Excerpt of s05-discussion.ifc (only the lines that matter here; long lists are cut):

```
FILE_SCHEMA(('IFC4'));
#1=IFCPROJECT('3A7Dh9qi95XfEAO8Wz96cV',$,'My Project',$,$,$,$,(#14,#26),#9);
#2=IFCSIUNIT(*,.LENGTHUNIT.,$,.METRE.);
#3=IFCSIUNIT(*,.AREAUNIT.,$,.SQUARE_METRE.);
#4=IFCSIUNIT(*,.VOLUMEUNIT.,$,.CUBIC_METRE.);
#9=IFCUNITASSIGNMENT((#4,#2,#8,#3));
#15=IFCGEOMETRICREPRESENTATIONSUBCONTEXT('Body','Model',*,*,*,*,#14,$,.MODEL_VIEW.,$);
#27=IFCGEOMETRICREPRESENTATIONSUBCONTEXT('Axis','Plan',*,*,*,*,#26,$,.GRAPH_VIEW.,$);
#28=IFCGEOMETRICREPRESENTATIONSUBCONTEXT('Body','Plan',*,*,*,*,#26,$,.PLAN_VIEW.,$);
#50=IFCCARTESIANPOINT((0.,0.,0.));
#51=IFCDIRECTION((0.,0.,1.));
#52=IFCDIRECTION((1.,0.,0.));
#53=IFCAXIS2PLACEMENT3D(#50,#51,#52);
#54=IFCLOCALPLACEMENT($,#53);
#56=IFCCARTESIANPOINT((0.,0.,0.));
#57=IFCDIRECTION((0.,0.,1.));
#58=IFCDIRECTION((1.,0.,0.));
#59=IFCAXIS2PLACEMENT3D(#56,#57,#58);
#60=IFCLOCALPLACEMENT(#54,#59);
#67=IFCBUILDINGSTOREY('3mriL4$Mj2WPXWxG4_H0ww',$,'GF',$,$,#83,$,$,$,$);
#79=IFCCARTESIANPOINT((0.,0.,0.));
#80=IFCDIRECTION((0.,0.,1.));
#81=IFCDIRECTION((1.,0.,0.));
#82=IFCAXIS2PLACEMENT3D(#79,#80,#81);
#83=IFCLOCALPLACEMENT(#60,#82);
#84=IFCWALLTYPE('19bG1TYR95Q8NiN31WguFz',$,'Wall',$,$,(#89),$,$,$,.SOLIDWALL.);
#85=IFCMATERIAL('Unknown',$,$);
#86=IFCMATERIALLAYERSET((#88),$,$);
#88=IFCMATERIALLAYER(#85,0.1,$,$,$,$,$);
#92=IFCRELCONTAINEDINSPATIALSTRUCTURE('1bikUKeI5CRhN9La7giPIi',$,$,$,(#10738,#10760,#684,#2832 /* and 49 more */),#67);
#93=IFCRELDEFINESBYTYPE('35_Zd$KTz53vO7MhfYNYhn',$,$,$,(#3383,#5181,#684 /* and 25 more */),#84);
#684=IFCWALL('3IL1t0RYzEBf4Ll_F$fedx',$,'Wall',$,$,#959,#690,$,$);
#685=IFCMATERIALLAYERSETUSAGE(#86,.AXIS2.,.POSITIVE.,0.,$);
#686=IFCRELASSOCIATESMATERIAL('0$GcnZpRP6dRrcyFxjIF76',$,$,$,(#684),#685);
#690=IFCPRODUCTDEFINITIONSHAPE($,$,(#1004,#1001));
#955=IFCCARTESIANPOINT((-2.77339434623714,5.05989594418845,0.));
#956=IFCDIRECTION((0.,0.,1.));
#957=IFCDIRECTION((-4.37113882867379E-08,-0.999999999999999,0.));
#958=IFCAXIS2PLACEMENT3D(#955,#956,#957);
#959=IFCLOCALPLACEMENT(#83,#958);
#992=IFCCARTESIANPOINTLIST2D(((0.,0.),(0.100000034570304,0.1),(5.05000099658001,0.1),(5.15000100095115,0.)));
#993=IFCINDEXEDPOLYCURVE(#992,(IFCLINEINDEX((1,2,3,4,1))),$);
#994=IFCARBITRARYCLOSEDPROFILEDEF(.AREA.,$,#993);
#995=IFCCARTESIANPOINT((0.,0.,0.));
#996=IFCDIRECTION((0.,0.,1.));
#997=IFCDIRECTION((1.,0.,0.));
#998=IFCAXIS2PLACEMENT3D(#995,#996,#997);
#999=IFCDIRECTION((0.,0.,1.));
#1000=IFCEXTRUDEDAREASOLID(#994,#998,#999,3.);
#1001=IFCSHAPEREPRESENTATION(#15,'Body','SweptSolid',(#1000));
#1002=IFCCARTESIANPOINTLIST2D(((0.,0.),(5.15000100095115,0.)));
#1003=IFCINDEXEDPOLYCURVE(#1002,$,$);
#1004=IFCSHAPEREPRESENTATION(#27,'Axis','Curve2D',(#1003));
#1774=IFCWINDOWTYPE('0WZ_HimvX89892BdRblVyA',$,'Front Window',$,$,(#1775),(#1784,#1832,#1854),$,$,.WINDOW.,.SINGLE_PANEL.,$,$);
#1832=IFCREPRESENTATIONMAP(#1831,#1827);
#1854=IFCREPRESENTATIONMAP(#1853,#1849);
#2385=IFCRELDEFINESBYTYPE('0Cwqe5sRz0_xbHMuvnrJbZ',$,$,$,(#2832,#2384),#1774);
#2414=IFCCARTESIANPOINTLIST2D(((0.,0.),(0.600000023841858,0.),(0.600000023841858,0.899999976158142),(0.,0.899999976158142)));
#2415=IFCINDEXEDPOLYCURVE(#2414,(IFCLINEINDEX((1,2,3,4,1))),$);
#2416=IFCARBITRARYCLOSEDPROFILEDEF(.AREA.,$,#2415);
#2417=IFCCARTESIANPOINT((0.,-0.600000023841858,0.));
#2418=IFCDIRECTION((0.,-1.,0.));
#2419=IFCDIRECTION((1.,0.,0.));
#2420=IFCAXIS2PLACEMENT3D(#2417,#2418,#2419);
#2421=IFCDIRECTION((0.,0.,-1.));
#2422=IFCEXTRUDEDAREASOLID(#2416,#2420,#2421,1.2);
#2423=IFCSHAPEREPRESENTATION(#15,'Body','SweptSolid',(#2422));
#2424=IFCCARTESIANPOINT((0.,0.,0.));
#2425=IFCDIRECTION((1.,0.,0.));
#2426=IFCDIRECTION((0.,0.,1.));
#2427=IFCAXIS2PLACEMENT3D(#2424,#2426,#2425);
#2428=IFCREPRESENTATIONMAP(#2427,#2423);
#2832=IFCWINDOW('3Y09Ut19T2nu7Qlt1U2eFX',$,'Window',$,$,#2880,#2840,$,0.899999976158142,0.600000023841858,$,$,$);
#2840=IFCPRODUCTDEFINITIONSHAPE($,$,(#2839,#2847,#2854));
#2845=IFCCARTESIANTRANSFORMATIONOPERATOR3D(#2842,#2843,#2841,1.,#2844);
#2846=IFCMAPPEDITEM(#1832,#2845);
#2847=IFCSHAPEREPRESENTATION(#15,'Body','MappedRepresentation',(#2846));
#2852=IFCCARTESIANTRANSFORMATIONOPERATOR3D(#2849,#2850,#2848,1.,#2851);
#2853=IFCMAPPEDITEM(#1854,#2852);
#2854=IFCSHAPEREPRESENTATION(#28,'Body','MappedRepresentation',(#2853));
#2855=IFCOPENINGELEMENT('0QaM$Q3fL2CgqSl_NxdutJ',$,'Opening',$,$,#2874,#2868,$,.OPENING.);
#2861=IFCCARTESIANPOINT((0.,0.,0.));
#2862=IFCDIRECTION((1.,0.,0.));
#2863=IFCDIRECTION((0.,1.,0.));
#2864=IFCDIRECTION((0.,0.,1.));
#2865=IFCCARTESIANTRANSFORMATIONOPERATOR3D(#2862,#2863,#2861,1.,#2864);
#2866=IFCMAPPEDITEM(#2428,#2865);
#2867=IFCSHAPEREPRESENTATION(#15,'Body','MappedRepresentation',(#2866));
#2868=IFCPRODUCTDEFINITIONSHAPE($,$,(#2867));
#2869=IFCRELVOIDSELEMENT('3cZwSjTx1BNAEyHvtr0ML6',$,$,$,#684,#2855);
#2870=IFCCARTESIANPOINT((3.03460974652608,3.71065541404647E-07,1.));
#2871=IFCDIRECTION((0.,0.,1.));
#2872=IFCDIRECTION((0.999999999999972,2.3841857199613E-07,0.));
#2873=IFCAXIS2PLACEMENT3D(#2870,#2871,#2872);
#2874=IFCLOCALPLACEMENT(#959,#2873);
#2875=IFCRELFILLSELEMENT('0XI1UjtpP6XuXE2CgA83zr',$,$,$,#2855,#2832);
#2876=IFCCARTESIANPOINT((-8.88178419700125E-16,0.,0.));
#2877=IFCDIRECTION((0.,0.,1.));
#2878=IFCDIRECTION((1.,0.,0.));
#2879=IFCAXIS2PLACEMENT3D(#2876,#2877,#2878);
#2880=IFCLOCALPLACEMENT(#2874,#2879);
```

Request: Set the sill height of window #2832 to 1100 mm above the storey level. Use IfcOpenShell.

```python
import numpy as np
import ifcopenshell
import ifcopenshell.api.geometry
import ifcopenshell.geom
import ifcopenshell.util.element
import ifcopenshell.util.placement
import ifcopenshell.util.shape
import ifcopenshell.util.unit

model = ifcopenshell.open("s05-discussion.ifc")
unit_scale = ifcopenshell.util.unit.calculate_unit_scale(model)

window = model.by_guid("3Y09Ut19T2nu7Qlt1U2eFX")
opening = window.FillsVoids[0].RelatingOpeningElement
storey = ifcopenshell.util.element.get_container(window, ifc_class="IfcBuildingStorey")
level = ifcopenshell.util.placement.get_local_placement(storey.ObjectPlacement)[2, 3]

# The opening's origin need not be at the sill, so measure its lowest point.
shape = ifcopenshell.geom.create_shape(ifcopenshell.geom.settings(), opening)
bottom = ifcopenshell.util.shape.get_shape_bottom_elevation(shape, shape.geometry) / unit_scale
dz = level + 1.1 - bottom

shift = np.array([0.0, 0.0, dz])
# The window is placed relative to its opening, so it follows when the opening moves.
matrix = ifcopenshell.util.placement.get_local_placement(opening.ObjectPlacement)
matrix[:3, 3] += shift
ifcopenshell.api.geometry.edit_object_placement(
    model, product=opening, matrix=matrix, is_si=False, should_transform_children=True
)

print(f"moved by {dz * unit_scale:+.3f} m")

model.write("s05-discussion_rev.ifc")
```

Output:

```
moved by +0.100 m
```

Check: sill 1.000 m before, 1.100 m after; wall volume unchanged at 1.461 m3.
